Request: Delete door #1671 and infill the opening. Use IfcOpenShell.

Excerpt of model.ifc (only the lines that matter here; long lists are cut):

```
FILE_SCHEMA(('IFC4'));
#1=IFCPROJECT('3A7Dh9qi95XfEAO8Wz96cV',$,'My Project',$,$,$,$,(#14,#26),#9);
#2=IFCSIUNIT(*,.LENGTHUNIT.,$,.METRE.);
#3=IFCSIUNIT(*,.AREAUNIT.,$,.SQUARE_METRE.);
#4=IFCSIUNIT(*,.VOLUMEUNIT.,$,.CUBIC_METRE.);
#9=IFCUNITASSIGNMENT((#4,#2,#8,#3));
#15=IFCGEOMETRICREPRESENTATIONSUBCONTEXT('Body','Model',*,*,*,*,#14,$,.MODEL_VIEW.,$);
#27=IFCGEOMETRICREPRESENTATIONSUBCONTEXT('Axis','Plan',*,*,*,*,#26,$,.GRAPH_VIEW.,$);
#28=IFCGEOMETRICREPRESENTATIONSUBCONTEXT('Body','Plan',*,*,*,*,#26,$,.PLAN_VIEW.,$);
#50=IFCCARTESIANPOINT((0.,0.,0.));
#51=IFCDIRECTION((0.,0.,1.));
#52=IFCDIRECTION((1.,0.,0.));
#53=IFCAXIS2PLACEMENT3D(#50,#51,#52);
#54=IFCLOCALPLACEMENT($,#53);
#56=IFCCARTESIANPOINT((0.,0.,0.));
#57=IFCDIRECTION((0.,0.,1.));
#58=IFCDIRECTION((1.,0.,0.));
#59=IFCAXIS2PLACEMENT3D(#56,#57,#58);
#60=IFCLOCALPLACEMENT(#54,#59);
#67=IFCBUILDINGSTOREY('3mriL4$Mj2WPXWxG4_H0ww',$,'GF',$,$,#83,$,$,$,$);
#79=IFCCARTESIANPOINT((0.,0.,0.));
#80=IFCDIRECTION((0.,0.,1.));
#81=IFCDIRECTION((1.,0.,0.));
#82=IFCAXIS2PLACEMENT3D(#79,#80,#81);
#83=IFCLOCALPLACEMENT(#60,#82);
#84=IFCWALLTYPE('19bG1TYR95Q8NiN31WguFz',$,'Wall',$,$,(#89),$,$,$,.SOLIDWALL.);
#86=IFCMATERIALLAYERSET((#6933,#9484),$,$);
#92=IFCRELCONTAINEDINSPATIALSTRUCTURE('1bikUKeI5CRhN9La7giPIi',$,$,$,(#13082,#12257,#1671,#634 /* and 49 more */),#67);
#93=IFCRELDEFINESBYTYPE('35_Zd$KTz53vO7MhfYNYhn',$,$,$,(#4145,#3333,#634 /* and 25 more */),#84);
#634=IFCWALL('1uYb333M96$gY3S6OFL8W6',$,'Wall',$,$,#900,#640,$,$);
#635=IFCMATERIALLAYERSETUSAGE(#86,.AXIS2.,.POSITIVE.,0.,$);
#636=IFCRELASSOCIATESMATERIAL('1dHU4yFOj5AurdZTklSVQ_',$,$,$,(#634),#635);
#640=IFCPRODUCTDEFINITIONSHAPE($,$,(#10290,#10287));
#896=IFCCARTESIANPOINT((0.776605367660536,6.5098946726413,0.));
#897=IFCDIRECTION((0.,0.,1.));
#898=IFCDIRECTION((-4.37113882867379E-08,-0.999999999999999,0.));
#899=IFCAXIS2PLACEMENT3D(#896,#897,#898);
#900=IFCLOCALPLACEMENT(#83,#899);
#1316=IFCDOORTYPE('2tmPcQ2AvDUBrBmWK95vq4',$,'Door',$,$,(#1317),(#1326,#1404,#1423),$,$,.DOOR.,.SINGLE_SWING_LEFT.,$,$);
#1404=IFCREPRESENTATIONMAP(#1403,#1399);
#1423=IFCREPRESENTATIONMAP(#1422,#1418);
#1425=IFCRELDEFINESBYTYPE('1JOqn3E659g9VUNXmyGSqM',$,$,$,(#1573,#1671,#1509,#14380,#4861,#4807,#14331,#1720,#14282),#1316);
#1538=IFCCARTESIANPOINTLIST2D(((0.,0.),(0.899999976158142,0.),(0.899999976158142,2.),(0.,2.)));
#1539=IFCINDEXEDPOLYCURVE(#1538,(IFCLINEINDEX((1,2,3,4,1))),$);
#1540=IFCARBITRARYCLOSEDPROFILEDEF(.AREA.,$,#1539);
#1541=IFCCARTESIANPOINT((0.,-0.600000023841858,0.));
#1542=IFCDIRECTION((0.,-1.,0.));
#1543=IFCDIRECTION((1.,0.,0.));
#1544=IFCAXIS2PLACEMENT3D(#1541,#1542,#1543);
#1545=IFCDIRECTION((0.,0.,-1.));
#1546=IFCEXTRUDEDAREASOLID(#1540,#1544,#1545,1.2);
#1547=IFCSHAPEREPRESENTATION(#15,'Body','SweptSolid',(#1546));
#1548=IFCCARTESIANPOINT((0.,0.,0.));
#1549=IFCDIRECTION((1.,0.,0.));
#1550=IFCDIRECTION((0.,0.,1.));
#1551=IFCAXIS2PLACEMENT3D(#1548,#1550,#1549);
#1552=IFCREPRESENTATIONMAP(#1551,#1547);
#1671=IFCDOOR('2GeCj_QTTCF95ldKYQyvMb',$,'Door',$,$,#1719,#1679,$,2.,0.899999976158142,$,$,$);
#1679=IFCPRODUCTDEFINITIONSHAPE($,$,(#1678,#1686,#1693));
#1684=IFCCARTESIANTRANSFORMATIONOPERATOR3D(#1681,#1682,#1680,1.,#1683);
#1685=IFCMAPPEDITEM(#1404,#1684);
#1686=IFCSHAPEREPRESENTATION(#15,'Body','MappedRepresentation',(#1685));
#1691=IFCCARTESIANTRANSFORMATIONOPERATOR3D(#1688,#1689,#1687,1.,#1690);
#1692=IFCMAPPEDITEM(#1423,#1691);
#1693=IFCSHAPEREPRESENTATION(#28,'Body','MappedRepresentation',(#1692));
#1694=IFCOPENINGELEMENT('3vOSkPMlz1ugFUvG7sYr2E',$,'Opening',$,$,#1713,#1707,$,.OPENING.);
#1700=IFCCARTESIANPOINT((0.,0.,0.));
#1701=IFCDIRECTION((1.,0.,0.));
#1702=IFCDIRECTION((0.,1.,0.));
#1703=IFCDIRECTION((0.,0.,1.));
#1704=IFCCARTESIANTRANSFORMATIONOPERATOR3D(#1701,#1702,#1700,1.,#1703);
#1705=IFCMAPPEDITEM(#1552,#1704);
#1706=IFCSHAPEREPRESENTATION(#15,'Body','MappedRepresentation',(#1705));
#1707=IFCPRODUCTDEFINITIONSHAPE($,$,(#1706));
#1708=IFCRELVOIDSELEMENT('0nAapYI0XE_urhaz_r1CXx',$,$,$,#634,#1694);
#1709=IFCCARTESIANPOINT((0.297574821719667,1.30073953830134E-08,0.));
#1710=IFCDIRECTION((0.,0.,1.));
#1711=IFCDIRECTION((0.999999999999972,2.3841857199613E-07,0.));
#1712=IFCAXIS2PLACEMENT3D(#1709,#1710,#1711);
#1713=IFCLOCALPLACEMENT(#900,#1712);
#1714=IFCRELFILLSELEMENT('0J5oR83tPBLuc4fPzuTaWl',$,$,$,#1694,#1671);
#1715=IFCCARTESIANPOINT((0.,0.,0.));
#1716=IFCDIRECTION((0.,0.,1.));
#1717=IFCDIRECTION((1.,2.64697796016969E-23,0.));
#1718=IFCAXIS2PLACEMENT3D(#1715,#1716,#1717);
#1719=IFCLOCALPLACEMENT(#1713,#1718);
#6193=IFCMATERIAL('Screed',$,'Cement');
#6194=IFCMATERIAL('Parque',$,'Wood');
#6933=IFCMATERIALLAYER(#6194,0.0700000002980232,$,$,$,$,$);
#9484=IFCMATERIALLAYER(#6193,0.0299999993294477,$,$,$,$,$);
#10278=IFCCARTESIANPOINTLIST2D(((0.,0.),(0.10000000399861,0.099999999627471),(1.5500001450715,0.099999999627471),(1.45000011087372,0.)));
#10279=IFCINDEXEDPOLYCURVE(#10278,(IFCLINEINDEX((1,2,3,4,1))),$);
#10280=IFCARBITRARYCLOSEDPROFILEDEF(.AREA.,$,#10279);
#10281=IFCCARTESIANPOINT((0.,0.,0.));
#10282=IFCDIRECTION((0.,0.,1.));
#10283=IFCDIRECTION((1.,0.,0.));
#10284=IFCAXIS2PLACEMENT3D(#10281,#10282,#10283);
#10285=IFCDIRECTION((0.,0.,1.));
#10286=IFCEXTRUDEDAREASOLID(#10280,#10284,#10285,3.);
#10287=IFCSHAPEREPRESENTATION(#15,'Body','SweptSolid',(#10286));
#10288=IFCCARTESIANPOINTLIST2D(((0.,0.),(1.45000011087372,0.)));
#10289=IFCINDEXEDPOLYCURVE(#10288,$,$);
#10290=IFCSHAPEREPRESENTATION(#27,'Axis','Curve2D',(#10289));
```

```python
import ifcopenshell
import ifcopenshell.api.feature
import ifcopenshell.api.root
import ifcopenshell.geom
import ifcopenshell.util.shape

model = ifcopenshell.open("model.ifc")
settings = ifcopenshell.geom.settings()


def volume(element):
    """Net volume in cubic metres, openings subtracted."""
    shape = ifcopenshell.geom.create_shape(settings, element)
    return ifcopenshell.util.shape.get_volume(shape.geometry)


door = model.by_guid("2GeCj_QTTCF95ldKYQyvMb")
opening = door.FillsVoids[0].RelatingOpeningElement
wall = opening.VoidsElements[0].RelatingBuildingElement
before = volume(wall)

ifcopenshell.api.root.remove_product(model, product=door)
ifcopenshell.api.feature.remove_feature(model, feature=opening)

after = volume(wall)

print(f"wall volume {before:.3f} -> {after:.3f} m3")

model.write("model_rev.ifc")
```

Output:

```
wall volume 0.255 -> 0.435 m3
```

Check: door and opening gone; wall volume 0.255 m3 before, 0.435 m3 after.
